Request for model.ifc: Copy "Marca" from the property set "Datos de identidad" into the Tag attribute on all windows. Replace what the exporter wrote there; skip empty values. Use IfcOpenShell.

First a look at what the model holds.

```python
import ifcopenshell
import ifcopenshell.util.element

model = ifcopenshell.open("model.ifc")
print(model.schema)
windows = model.by_type("IfcWindow")
print(len(windows), "windows")
for e in windows[:8]:
    source = ifcopenshell.util.element.get_pset(e, "Datos de identidad", "Marca")
    target = e.Tag
    print(e.id(), repr(source), repr(target), sep=" | ")
```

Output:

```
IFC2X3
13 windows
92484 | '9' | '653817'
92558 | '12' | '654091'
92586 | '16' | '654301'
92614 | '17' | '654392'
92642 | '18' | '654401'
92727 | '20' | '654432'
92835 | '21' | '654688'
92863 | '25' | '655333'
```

```python
import ifcopenshell
import ifcopenshell.util.element

model = ifcopenshell.open("model.ifc")

count = 0
for e in model.by_type("IfcWindow"):
    value = ifcopenshell.util.element.get_pset(e, "Datos de identidad", "Marca")
    current = e.Tag
    if not value or not value.strip() or current == value:
        continue
    e.Tag = value
    count += 1

print(count, "windows updated")

model.write("model_edited.ifc")
```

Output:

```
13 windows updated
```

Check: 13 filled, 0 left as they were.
